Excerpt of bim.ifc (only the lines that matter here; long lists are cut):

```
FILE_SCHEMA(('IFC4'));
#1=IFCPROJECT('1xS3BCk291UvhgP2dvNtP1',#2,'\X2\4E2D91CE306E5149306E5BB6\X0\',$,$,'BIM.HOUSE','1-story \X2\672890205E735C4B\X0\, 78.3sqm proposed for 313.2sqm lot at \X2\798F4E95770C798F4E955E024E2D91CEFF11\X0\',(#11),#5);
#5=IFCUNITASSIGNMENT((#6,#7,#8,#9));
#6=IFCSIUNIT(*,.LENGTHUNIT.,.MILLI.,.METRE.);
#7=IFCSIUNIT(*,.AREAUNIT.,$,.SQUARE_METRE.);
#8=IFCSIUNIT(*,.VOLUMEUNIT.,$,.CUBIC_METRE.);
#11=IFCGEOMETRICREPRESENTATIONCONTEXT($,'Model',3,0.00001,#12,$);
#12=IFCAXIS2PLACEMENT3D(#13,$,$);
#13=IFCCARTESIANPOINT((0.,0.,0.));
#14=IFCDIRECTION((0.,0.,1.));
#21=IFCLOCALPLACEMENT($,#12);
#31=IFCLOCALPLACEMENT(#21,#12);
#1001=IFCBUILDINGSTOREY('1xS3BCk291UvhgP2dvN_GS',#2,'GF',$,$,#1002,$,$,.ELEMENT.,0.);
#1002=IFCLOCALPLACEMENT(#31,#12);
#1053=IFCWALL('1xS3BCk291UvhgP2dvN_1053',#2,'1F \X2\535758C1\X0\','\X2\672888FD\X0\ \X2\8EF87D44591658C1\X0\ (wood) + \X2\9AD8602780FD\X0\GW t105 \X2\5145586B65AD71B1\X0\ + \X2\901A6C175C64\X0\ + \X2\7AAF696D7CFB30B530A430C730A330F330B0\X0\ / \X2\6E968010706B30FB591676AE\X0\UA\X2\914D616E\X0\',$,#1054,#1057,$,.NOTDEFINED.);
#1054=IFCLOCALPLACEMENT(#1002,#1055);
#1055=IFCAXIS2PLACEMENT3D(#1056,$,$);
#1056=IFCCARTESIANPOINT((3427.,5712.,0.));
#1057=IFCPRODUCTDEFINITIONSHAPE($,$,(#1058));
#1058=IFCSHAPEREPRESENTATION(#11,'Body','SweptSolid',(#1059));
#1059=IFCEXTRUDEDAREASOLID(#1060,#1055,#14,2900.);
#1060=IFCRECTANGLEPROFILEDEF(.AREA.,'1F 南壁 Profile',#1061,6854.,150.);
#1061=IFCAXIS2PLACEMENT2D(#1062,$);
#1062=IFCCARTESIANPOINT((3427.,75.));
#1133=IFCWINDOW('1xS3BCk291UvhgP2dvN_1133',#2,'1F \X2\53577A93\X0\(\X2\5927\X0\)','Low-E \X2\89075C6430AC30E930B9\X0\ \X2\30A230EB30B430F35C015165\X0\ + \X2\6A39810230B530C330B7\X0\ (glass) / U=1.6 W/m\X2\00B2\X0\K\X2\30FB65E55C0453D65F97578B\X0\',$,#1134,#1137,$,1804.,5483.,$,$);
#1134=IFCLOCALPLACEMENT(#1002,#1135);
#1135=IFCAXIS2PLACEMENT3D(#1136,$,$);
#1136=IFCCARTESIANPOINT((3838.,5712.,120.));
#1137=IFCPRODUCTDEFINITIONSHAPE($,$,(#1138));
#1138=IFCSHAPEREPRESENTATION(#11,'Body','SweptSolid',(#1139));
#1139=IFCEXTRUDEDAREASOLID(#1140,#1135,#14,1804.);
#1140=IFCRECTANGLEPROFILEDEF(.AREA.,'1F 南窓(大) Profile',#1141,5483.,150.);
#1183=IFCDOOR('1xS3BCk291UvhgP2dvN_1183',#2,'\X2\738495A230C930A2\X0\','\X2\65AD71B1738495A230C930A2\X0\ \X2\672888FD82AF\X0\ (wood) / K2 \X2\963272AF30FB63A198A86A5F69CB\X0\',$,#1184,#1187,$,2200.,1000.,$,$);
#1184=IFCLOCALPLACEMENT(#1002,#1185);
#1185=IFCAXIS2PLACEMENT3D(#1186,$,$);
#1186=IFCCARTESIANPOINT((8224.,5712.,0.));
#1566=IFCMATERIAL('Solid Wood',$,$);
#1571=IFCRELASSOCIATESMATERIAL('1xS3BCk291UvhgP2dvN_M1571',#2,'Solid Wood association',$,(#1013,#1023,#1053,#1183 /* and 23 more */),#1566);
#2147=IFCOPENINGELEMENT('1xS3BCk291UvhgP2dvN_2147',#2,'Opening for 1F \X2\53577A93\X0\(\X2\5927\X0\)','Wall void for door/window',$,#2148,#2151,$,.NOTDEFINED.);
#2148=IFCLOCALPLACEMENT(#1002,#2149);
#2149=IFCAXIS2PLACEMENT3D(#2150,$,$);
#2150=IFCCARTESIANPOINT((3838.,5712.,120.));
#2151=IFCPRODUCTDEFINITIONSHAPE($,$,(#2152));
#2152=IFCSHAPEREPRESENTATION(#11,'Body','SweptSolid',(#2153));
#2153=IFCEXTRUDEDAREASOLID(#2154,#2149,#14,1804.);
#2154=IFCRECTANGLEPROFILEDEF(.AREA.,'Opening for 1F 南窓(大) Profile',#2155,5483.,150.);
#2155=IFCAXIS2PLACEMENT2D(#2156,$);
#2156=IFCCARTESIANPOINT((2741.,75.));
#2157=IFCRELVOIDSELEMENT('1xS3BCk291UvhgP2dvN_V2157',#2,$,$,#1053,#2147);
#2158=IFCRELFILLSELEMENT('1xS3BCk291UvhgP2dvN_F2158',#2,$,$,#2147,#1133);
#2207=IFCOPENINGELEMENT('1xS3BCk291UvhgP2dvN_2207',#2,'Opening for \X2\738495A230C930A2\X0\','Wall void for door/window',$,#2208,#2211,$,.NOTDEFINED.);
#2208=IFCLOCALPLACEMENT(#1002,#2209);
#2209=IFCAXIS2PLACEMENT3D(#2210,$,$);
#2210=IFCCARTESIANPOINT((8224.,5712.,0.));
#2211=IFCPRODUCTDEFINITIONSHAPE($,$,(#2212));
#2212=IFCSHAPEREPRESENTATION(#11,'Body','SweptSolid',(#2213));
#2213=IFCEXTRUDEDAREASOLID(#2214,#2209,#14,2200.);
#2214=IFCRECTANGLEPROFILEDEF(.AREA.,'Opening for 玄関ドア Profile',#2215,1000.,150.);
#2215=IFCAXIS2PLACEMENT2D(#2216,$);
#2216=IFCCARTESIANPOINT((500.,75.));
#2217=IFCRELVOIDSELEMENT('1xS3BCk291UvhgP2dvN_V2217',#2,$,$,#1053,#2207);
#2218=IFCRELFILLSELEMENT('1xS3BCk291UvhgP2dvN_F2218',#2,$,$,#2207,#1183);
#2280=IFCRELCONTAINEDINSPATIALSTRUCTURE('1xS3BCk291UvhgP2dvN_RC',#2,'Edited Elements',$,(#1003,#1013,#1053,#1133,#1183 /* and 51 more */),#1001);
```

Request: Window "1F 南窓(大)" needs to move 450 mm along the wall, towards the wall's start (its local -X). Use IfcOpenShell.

```python
import ifcopenshell
import ifcopenshell.api.geometry
import ifcopenshell.util.placement

model = ifcopenshell.open("bim.ifc")

window = model.by_guid("1xS3BCk291UvhgP2dvN_1133")
opening = window.FillsVoids[0].RelatingOpeningElement
wall = opening.VoidsElements[0].RelatingBuildingElement

wall_matrix = ifcopenshell.util.placement.get_local_placement(wall.ObjectPlacement)
shift = wall_matrix[:3, 0] * -450.0
before = ifcopenshell.util.placement.get_local_placement(window.ObjectPlacement)[:3, 3].copy()

# The window is not placed relative to its opening, so move both.
for product in (opening, window):
    matrix = ifcopenshell.util.placement.get_local_placement(product.ObjectPlacement)
    matrix[:3, 3] += shift
    ifcopenshell.api.geometry.edit_object_placement(model, product=product, matrix=matrix, is_si=False)

after = ifcopenshell.util.placement.get_local_placement(window.ObjectPlacement)[:3, 3]
print("window moved by", (after - before).round(3) + 0.0)

model.write("bim_v2.ifc")
```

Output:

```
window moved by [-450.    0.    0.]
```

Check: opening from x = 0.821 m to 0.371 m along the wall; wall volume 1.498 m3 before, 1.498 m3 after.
